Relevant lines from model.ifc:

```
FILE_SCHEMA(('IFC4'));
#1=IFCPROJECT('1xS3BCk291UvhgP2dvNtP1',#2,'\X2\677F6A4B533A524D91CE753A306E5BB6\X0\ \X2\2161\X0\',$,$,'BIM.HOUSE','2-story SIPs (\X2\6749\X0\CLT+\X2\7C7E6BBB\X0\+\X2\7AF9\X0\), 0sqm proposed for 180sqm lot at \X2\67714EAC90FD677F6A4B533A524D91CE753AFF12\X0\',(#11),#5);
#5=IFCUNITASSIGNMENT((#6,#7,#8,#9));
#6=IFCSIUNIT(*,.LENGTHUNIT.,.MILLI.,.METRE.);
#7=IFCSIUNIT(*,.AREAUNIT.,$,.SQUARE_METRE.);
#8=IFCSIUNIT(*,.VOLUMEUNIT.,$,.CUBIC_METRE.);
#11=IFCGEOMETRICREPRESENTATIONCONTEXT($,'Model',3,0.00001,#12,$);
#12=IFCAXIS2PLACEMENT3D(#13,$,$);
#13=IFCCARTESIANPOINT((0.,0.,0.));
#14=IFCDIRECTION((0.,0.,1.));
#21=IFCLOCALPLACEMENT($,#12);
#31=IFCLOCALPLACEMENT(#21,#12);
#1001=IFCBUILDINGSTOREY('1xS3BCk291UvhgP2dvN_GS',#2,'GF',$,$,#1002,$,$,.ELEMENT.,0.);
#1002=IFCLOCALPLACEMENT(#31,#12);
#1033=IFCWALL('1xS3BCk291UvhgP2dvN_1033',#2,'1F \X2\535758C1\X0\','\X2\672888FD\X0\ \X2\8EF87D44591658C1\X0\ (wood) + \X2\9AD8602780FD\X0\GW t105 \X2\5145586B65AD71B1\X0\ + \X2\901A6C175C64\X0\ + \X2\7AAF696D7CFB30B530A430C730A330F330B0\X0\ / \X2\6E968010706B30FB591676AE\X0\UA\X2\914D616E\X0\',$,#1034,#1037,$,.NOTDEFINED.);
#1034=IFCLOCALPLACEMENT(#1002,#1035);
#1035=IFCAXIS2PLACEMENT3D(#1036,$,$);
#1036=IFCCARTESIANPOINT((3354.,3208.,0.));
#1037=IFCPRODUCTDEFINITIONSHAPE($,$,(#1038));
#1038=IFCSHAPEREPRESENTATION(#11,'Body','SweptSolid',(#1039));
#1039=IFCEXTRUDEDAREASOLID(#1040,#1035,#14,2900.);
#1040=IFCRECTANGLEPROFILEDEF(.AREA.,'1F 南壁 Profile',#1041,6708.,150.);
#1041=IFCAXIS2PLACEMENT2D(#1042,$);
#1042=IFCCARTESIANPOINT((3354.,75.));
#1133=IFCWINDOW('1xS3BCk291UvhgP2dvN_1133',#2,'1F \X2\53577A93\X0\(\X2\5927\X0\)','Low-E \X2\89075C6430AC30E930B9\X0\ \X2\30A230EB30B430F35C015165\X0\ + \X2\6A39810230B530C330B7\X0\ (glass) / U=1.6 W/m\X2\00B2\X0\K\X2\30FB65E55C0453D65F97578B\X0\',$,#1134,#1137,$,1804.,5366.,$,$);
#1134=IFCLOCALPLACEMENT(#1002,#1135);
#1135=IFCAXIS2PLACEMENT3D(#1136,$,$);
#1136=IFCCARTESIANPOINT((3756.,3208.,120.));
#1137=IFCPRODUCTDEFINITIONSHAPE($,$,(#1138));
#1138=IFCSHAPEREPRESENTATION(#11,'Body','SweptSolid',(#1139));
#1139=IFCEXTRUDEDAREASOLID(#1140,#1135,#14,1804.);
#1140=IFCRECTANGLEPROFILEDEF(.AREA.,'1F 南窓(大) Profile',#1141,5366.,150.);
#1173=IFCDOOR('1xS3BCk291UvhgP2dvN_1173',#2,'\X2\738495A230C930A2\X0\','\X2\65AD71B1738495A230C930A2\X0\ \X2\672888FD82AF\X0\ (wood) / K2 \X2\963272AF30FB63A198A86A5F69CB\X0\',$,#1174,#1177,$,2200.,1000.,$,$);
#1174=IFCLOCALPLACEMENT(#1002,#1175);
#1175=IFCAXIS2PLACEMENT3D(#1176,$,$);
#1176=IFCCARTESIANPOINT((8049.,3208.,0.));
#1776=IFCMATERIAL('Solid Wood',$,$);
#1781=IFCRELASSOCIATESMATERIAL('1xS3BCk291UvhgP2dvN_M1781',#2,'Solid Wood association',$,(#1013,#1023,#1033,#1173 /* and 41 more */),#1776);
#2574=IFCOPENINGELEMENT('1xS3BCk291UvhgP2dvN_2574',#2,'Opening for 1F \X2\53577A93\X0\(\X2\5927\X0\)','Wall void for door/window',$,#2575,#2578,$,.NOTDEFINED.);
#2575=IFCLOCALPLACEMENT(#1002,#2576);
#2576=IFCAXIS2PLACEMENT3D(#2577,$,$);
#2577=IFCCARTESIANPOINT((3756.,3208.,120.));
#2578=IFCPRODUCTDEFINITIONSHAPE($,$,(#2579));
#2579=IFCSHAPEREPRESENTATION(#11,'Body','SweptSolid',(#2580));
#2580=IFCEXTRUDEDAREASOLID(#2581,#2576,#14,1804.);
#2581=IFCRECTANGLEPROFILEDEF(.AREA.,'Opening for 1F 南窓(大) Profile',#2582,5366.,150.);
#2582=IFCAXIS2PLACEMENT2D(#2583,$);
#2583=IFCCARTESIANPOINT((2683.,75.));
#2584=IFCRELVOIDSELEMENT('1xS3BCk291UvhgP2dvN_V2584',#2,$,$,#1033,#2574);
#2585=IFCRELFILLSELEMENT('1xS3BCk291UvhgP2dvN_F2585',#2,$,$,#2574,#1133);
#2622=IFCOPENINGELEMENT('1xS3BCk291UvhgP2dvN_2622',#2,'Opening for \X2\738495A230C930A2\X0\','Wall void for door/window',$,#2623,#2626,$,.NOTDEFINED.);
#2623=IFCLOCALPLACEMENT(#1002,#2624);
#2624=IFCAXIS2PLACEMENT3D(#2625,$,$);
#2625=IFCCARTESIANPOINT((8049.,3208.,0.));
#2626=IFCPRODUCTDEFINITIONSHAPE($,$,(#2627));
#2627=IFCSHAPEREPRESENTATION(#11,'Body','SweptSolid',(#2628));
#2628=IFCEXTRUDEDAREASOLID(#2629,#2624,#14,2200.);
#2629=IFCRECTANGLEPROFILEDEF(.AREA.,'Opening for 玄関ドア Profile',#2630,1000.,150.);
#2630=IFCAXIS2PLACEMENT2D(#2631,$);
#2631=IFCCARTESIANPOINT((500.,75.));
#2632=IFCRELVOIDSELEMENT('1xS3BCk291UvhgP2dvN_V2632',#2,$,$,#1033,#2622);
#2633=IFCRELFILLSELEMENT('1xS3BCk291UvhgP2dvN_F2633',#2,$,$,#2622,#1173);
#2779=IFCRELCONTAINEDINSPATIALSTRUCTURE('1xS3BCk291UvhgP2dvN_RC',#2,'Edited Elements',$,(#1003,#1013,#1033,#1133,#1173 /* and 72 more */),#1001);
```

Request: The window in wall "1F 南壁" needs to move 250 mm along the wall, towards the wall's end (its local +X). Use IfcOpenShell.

```python
import ifcopenshell
import ifcopenshell.api.geometry
import ifcopenshell.util.placement
import ifcopenshell.util.unit

model = ifcopenshell.open("model.ifc")
unit_scale = ifcopenshell.util.unit.calculate_unit_scale(model)

window = model.by_id(1133)
opening = window.FillsVoids[0].RelatingOpeningElement
wall = opening.VoidsElements[0].RelatingBuildingElement

wall_matrix = ifcopenshell.util.placement.get_local_placement(wall.ObjectPlacement)
shift = wall_matrix[:3, 0] * 0.25 / unit_scale
before = ifcopenshell.util.placement.get_local_placement(window.ObjectPlacement)[:3, 3].copy()

# The window is not placed relative to its opening, so move both.
for product in (opening, window):
    matrix = ifcopenshell.util.placement.get_local_placement(product.ObjectPlacement)
    matrix[:3, 3] += shift
    ifcopenshell.api.geometry.edit_object_placement(model, product=product, matrix=matrix, is_si=False)

after = ifcopenshell.util.placement.get_local_placement(window.ObjectPlacement)[:3, 3]
print("window moved by", (after - before).round(3) + 0.0)

model.write("model_rev.ifc")
```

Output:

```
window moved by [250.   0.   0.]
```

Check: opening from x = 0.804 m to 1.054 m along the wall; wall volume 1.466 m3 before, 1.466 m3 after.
